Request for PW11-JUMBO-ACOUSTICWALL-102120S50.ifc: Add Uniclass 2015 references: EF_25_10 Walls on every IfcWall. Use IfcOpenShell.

First a look at what the model holds.

```python
import ifcopenshell

model = ifcopenshell.open("PW11-JUMBO-ACOUSTICWALL-102120S50.ifc")
print(model.schema)
print("classifications:", [c.Name for c in model.by_type("IfcClassification")])
for ifc_class in ("IfcDoor", "IfcRoof", "IfcStair", "IfcWall", "IfcWindow"):
    print(ifc_class, len(model.by_type(ifc_class)))
```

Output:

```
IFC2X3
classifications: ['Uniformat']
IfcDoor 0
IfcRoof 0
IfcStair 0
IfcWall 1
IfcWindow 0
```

```python
import ifcopenshell
import ifcopenshell.api.classification

model = ifcopenshell.open("PW11-JUMBO-ACOUSTICWALL-102120S50.ifc")

# IFC2X3 requires Source and Edition and has no link from the project to the system.
system = model.create_entity("IfcClassification", Source="NBS", Edition="2015", Name="Uniclass 2015")

codes = {
    "IfcWall": ("EF_25_10", "Walls"),
}
for ifc_class, (code, name) in codes.items():
    products = model.by_type(ifc_class)
    ifcopenshell.api.classification.add_reference(
        model, products=products, classification=system, identification=code, name=name
    )
    print(code, len(products))

model.write("PW11-JUMBO-ACOUSTICWALL-102120S50_rev.ifc")
```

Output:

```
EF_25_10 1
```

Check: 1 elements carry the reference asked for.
